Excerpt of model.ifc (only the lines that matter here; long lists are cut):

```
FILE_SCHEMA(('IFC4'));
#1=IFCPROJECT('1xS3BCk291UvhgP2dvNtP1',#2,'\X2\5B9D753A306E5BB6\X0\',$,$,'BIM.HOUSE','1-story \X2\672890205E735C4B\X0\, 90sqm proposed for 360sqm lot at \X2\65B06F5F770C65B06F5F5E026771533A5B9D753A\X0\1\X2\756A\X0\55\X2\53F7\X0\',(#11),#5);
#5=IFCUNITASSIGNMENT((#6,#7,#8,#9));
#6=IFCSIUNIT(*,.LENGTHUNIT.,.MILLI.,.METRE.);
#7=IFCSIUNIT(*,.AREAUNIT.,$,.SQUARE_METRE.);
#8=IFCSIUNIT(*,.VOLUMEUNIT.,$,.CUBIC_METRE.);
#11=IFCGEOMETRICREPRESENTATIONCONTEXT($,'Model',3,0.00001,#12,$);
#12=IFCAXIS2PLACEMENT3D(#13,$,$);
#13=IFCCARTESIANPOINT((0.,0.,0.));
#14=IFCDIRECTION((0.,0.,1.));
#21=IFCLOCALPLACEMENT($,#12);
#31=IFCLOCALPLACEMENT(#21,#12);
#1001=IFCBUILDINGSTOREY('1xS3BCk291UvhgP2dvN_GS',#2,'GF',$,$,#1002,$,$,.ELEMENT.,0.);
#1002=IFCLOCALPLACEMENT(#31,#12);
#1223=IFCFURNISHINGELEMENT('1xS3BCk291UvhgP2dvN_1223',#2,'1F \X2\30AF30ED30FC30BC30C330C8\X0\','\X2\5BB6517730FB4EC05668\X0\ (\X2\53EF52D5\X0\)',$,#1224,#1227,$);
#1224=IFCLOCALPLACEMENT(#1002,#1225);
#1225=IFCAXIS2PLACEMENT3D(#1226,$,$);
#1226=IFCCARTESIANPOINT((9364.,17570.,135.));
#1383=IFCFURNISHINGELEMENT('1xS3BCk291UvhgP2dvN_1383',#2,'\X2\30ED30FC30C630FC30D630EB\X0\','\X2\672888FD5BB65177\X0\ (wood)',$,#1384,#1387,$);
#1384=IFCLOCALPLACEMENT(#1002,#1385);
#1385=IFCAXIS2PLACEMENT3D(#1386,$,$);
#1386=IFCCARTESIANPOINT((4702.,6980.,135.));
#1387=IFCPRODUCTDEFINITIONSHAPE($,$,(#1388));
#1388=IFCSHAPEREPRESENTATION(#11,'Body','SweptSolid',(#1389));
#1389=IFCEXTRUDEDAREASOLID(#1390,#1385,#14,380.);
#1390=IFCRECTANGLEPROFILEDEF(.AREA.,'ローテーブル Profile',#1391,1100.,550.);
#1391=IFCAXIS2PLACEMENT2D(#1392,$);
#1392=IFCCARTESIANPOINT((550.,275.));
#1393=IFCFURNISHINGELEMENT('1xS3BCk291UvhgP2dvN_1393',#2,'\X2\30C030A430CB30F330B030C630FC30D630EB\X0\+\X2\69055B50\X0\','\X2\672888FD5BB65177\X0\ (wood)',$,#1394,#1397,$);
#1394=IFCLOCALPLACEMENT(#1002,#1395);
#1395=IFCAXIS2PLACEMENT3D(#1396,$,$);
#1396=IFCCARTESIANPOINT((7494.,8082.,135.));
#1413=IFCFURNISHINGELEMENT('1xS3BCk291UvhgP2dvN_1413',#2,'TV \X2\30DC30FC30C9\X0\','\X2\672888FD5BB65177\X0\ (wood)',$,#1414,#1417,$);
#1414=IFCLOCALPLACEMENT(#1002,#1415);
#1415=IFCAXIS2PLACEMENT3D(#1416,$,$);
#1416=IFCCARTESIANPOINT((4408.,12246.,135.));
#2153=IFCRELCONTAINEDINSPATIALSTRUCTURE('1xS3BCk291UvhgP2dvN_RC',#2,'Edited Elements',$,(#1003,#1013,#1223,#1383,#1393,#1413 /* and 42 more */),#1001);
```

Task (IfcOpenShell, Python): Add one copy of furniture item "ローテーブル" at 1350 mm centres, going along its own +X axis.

```python
import ifcopenshell
import ifcopenshell.api.geometry
import ifcopenshell.api.root
import ifcopenshell.util.element
import ifcopenshell.util.placement
import ifcopenshell.util.unit

model = ifcopenshell.open("model.ifc")
unit_scale = ifcopenshell.util.unit.calculate_unit_scale(model)


def reuse_history(source, copy):
    """copy_class also copies each property set's owner history, people and application; keep the originals."""
    for rel in copy.IsDefinedBy:
        if rel.is_a("IfcRelDefinesByProperties") and (history := rel.RelatingPropertyDefinition.OwnerHistory):
            rel.RelatingPropertyDefinition.OwnerHistory = source.OwnerHistory
            ifcopenshell.util.element.remove_deep2(model, history)


source = model.by_guid("1xS3BCk291UvhgP2dvN_1383")
base = ifcopenshell.util.placement.get_local_placement(source.ObjectPlacement)
step = base[:3, 0] * 1.35 / unit_scale

for i in range(1, 2):
    copy = ifcopenshell.api.root.copy_class(model, product=source)
    copy.Representation = ifcopenshell.util.element.copy_deep(
        model, source.Representation, exclude=["IfcGeometricRepresentationContext", "IfcRepresentationMap"]
    )
    reuse_history(source, copy)
    matrix = base.copy()
    matrix[:3, 3] += i * step
    print("added at", matrix[:3, 3].round(3) + 0.0)
    ifcopenshell.api.geometry.edit_object_placement(model, product=copy, matrix=matrix, is_si=False)

model.write("model_v2.ifc")
```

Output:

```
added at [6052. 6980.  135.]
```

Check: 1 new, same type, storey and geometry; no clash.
